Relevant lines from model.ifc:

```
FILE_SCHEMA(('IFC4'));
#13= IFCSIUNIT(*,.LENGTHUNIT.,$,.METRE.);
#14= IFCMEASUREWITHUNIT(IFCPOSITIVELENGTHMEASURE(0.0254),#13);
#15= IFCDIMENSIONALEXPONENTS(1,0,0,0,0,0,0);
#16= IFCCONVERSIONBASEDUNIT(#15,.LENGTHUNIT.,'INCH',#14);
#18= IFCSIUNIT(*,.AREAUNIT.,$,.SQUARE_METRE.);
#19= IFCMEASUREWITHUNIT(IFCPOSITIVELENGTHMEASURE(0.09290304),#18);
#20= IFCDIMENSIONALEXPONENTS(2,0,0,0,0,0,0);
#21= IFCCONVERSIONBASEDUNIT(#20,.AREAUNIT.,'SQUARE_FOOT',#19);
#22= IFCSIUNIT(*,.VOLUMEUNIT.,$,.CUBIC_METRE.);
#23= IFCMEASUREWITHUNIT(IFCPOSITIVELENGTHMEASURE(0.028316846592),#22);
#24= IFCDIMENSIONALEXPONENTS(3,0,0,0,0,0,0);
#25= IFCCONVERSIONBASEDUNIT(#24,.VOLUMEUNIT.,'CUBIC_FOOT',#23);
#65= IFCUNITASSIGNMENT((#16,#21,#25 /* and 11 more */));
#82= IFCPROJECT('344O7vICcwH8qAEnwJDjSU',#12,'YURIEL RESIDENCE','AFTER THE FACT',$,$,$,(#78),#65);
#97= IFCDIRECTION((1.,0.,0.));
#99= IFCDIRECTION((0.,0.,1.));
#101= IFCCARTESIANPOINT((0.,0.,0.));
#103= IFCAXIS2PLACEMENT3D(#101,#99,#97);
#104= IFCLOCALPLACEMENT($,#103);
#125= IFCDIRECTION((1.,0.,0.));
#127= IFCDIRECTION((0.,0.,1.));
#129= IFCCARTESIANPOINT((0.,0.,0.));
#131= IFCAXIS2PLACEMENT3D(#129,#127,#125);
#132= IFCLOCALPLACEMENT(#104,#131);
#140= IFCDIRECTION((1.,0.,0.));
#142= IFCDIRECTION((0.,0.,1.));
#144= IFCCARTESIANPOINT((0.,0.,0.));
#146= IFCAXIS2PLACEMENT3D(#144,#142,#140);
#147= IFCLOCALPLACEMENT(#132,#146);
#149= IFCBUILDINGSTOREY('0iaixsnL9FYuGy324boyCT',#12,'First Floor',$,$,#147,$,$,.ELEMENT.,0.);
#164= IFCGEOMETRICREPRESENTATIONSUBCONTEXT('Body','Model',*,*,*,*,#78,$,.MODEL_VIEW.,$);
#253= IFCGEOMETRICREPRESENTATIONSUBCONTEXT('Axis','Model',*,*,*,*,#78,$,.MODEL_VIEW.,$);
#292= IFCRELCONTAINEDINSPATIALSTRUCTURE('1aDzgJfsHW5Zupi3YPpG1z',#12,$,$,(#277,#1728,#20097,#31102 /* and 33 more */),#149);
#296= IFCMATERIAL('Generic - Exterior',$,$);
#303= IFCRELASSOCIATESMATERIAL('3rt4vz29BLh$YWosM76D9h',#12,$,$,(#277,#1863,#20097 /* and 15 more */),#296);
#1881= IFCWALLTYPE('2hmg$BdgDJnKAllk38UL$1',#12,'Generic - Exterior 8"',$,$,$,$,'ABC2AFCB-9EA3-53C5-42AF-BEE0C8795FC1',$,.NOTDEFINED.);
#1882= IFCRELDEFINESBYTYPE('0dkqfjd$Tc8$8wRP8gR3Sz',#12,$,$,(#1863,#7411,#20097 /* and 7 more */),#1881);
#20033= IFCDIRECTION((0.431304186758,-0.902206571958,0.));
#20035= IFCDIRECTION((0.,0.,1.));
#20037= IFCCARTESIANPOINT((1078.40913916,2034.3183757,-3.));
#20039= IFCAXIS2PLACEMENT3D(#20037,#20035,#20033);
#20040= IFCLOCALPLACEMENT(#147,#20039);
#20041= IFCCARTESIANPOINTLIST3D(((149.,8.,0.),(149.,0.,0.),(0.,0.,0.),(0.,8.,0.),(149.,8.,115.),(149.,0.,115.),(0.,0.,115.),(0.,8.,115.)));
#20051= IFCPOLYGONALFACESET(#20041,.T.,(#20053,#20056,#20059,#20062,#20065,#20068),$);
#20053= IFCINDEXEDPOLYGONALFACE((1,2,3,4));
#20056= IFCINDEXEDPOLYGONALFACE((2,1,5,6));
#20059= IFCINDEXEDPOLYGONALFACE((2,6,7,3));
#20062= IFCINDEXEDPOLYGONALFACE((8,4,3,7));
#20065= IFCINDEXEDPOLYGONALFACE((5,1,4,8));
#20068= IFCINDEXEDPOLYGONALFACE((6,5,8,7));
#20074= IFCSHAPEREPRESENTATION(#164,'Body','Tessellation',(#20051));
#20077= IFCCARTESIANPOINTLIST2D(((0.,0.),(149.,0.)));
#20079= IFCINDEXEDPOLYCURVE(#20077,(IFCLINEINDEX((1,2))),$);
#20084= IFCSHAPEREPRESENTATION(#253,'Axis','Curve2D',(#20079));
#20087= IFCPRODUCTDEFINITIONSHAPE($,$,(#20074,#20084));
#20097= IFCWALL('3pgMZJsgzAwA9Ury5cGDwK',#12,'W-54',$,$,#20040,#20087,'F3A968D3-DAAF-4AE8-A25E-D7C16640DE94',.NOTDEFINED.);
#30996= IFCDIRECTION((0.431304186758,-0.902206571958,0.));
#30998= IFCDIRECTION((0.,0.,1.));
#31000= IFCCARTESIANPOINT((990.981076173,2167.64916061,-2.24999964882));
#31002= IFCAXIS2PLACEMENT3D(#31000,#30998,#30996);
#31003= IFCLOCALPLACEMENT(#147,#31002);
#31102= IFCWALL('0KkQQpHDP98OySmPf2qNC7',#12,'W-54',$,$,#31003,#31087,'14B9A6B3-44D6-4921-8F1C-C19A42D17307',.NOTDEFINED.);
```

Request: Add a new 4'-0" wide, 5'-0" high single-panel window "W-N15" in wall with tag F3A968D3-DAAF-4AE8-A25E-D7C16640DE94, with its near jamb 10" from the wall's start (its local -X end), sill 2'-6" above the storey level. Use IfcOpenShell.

```python
import numpy as np
import ifcopenshell
import ifcopenshell.api.feature
import ifcopenshell.api.geometry
import ifcopenshell.api.root
import ifcopenshell.api.spatial
import ifcopenshell.geom
import ifcopenshell.util.element
import ifcopenshell.util.placement
import ifcopenshell.util.representation
import ifcopenshell.util.shape
import ifcopenshell.util.unit

model = ifcopenshell.open("model.ifc")
unit_scale = ifcopenshell.util.unit.calculate_unit_scale(model)
settings = ifcopenshell.geom.settings()


def volume(element):
    """Net volume in cubic metres, openings subtracted."""
    shape = ifcopenshell.geom.create_shape(settings, element)
    return ifcopenshell.util.shape.get_volume(shape.geometry)


wall = model.by_guid("3pgMZJsgzAwA9Ury5cGDwK")
storey = ifcopenshell.util.element.get_container(wall, ifc_class="IfcBuildingStorey")
context = ifcopenshell.util.representation.get_context(model, "Model", "Body", "MODEL_VIEW")
before = volume(wall)

width, height, from_end, sill = 1.2192, 1.524, 0.254, 0.762  # metres

# The wall runs along its own X axis, and the end named is its -X end.
wall_shape = ifcopenshell.geom.create_shape(settings, wall)
x, y, z = ifcopenshell.util.shape.get_vertices(wall_shape.geometry).T
start = x.min() + from_end
face, thickness = float(y.min()), float(y.max() - y.min())
wall_matrix = ifcopenshell.util.placement.get_local_placement(wall.ObjectPlacement)
level = ifcopenshell.util.placement.get_local_placement(storey.ObjectPlacement)[2, 3]


def in_wall(x, y):
    """Placement at x, y metres in the wall's axes, at sill height."""
    matrix = wall_matrix.copy()
    matrix[:, 3] = wall_matrix @ np.array([x / unit_scale, y / unit_scale, 0.0, 1.0])
    matrix[2, 3] = level + sill / unit_scale
    return matrix


# Opening: a box that overshoots both wall faces by 50 mm.
opening = ifcopenshell.api.root.create_entity(model, ifc_class="IfcOpeningElement", predefined_type="OPENING")
box = ifcopenshell.api.geometry.add_wall_representation(
    model, context=context, length=width, height=height, thickness=thickness + 0.1
)
ifcopenshell.api.geometry.assign_representation(model, product=opening, representation=box)
ifcopenshell.api.geometry.edit_object_placement(model, product=opening, matrix=in_wall(start, face - 0.05), is_si=False)
ifcopenshell.api.feature.add_feature(model, feature=opening, element=wall)

window = ifcopenshell.api.root.create_entity(model, ifc_class="IfcWindow", name="W-N15", predefined_type="WINDOW")
window.OverallWidth, window.OverallHeight = width / unit_scale, height / unit_scale
window.PartitioningType = "SINGLE_PANEL"
body = ifcopenshell.api.geometry.add_window_representation(
    model,
    context=context,
    overall_width=window.OverallWidth,
    overall_height=window.OverallHeight,
    partition_type="SINGLE_PANEL",
)
ifcopenshell.api.geometry.assign_representation(model, product=window, representation=body)
ifcopenshell.api.spatial.assign_container(model, products=[window], relating_structure=storey)
ifcopenshell.api.feature.add_filling(model, opening=opening, element=window)

# Centre the window in the wall's thickness.
ifcopenshell.api.geometry.edit_object_placement(model, product=window, matrix=in_wall(start, face), is_si=False)
window_shape = ifcopenshell.geom.create_shape(settings, window)
depth = ifcopenshell.util.shape.get_vertices(window_shape.geometry)[:, 1]
offset = face + thickness / 2 - (depth.min() + depth.max()) / 2
ifcopenshell.api.geometry.edit_object_placement(model, product=window, matrix=in_wall(start, offset), is_si=False)

after = volume(wall)

print(f"wall volume {before:.3f} -> {after:.3f} m3")

model.write("model_updated.ifc")
```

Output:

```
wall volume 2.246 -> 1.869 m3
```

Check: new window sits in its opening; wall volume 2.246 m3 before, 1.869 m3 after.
